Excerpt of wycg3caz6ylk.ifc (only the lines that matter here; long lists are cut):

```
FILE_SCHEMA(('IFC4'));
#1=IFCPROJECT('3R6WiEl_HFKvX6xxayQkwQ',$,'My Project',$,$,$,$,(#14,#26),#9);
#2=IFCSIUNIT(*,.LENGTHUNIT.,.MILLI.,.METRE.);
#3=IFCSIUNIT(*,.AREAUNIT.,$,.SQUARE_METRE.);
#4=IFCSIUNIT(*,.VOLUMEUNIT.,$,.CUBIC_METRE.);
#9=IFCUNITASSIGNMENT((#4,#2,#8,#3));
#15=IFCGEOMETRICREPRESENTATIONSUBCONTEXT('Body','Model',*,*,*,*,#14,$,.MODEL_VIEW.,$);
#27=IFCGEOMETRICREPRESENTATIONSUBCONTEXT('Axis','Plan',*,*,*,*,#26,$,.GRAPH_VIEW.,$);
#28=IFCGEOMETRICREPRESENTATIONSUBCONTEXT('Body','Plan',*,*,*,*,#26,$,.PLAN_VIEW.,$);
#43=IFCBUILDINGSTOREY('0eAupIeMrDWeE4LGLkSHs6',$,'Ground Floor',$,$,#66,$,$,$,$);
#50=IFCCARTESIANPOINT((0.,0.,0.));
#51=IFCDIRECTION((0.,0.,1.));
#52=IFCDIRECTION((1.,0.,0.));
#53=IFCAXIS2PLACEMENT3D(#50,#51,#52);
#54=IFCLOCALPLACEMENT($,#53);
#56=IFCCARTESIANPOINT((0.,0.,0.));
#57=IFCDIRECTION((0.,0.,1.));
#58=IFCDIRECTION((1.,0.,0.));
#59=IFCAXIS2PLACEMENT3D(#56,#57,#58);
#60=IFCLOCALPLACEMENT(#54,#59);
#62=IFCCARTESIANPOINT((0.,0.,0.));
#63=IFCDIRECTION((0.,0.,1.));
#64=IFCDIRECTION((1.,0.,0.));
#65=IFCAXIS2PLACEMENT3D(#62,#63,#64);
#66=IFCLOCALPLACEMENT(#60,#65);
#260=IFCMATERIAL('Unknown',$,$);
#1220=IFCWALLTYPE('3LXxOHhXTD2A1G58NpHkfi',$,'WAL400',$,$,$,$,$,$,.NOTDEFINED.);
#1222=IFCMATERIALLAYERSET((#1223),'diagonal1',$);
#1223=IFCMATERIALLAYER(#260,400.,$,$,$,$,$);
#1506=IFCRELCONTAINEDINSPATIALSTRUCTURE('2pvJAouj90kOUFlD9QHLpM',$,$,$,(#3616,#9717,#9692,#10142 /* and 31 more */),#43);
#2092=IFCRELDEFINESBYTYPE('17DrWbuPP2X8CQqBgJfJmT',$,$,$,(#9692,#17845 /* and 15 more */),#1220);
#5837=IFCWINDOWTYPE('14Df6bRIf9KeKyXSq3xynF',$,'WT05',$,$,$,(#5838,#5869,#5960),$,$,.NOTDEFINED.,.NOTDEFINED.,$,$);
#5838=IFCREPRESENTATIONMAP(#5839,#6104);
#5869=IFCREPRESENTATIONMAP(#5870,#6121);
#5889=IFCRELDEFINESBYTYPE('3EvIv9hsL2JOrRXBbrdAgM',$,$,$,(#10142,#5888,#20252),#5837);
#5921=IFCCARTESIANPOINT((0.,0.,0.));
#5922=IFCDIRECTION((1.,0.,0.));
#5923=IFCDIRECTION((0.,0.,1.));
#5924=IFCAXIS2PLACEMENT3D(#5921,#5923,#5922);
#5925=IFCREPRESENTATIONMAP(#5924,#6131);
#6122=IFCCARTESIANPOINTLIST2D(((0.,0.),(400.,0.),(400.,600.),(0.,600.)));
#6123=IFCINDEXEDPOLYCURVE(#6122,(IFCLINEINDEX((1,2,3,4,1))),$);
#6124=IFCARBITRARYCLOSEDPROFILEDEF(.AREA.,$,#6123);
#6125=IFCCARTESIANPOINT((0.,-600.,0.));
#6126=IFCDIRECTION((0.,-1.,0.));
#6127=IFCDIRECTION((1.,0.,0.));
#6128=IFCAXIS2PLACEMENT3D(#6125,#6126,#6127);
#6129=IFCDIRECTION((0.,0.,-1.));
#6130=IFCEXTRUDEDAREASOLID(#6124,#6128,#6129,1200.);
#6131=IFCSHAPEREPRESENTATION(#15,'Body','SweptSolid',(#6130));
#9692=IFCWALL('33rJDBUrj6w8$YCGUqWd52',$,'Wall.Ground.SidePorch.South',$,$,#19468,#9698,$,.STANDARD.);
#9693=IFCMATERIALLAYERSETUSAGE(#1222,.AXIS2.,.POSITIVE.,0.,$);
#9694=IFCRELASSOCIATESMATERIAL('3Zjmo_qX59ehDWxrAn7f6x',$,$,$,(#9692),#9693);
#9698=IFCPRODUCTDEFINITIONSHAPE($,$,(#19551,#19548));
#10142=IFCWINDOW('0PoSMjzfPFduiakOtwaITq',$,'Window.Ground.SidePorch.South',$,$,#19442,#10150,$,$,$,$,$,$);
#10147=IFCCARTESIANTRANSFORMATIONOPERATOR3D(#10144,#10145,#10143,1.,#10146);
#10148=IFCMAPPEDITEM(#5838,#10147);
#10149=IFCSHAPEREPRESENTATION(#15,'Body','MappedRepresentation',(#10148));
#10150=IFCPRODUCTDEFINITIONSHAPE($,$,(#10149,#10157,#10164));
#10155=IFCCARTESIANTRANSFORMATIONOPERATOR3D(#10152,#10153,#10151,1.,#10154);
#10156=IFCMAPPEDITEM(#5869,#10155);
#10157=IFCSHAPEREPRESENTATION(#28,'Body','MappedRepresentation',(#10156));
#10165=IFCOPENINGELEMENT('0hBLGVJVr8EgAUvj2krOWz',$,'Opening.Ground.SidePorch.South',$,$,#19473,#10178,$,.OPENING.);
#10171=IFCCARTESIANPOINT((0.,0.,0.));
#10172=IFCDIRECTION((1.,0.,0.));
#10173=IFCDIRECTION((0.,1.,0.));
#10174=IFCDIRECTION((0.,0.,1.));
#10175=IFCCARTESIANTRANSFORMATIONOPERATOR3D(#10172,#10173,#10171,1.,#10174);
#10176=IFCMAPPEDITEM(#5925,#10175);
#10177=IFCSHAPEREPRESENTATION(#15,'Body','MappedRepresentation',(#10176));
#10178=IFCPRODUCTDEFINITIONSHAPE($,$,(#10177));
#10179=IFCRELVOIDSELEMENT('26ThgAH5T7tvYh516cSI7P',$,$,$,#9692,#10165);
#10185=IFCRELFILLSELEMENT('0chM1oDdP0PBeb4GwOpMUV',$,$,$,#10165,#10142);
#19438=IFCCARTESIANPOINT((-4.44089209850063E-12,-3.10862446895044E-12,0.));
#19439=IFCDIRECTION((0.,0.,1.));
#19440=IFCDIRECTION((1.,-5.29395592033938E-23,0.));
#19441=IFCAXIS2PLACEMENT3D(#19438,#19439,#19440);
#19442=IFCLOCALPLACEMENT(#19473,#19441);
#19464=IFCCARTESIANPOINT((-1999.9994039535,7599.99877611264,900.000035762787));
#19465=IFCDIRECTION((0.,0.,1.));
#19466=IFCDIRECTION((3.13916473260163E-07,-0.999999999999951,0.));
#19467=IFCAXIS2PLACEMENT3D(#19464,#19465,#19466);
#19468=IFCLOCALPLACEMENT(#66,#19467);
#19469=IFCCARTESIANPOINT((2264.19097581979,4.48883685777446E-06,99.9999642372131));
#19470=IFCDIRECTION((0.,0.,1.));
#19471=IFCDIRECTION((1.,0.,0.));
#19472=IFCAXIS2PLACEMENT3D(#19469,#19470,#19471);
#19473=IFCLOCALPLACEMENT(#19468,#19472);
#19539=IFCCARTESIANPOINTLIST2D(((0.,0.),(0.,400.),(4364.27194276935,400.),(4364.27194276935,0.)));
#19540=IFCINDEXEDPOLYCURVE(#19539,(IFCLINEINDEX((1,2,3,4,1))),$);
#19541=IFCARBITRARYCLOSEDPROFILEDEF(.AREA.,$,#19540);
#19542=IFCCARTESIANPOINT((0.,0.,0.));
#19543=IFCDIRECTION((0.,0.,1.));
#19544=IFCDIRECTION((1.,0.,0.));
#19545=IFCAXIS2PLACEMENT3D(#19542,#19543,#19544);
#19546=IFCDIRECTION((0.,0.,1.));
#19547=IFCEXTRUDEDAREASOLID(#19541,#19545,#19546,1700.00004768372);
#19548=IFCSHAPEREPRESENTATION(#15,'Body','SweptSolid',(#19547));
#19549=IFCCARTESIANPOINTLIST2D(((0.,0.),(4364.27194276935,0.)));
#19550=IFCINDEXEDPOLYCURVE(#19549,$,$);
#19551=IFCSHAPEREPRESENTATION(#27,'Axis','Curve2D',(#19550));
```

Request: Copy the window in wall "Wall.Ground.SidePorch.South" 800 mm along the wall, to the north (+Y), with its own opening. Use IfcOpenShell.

```python
import ifcopenshell
import ifcopenshell.api.feature
import ifcopenshell.api.geometry
import ifcopenshell.api.root
import ifcopenshell.geom
import ifcopenshell.util.element
import ifcopenshell.util.placement
import ifcopenshell.util.shape

model = ifcopenshell.open("wycg3caz6ylk.ifc")
settings = ifcopenshell.geom.settings()


def volume(element):
    """Net volume in cubic metres, openings subtracted."""
    shape = ifcopenshell.geom.create_shape(settings, element)
    return ifcopenshell.util.shape.get_volume(shape.geometry)


window = model.by_guid("0PoSMjzfPFduiakOtwaITq")
opening = window.FillsVoids[0].RelatingOpeningElement
wall = opening.VoidsElements[0].RelatingBuildingElement
before = volume(wall)
shift = ifcopenshell.util.placement.get_local_placement(wall.ObjectPlacement)[:3, 0] * -800.0

# copy_class copies the void relationship, type, container and properties, but no geometry.
new_opening = ifcopenshell.api.root.copy_class(model, product=opening)
new_opening.Representation = ifcopenshell.util.element.copy_deep(
    model, opening.Representation, exclude=["IfcGeometricRepresentationContext", "IfcRepresentationMap"]
)
new_window = ifcopenshell.api.root.copy_class(model, product=window)
new_window.Representation = ifcopenshell.util.element.copy_deep(
    model, window.Representation, exclude=["IfcGeometricRepresentationContext", "IfcRepresentationMap"]
)
ifcopenshell.api.feature.add_filling(model, opening=new_opening, element=new_window)

for old, new in ((opening, new_opening), (window, new_window)):
    matrix = ifcopenshell.util.placement.get_local_placement(old.ObjectPlacement)
    matrix[:3, 3] += shift
    ifcopenshell.api.geometry.edit_object_placement(model, product=new, matrix=matrix, is_si=False)

after = volume(wall)

print(f"wall volume {before:.3f} -> {after:.3f} m3")

model.write("wycg3caz6ylk_rev.ifc")
```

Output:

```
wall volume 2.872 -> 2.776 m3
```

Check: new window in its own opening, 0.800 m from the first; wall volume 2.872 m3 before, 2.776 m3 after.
